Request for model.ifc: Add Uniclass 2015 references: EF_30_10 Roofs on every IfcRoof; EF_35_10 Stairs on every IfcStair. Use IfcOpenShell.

First a look at what the model holds.

```python
import ifcopenshell

model = ifcopenshell.open("model.ifc")
print(model.schema)
print("classifications:", [c.Name for c in model.by_type("IfcClassification")])
for ifc_class in ("IfcDoor", "IfcRoof", "IfcStair", "IfcWall", "IfcWindow"):
    print(ifc_class, len(model.by_type(ifc_class)))
```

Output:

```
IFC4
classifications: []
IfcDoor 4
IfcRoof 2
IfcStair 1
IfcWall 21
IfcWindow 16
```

```python
import ifcopenshell
import ifcopenshell.api.classification

model = ifcopenshell.open("model.ifc")

system = ifcopenshell.api.classification.add_classification(model, classification="Uniclass 2015")

codes = {
    "IfcRoof": ("EF_30_10", "Roofs"),
    "IfcStair": ("EF_35_10", "Stairs"),
}
for ifc_class, (code, name) in codes.items():
    products = model.by_type(ifc_class)
    ifcopenshell.api.classification.add_reference(
        model, products=products, classification=system, identification=code, name=name
    )
    print(code, len(products))

model.write("model-out.ifc")
```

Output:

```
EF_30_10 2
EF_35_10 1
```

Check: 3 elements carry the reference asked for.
